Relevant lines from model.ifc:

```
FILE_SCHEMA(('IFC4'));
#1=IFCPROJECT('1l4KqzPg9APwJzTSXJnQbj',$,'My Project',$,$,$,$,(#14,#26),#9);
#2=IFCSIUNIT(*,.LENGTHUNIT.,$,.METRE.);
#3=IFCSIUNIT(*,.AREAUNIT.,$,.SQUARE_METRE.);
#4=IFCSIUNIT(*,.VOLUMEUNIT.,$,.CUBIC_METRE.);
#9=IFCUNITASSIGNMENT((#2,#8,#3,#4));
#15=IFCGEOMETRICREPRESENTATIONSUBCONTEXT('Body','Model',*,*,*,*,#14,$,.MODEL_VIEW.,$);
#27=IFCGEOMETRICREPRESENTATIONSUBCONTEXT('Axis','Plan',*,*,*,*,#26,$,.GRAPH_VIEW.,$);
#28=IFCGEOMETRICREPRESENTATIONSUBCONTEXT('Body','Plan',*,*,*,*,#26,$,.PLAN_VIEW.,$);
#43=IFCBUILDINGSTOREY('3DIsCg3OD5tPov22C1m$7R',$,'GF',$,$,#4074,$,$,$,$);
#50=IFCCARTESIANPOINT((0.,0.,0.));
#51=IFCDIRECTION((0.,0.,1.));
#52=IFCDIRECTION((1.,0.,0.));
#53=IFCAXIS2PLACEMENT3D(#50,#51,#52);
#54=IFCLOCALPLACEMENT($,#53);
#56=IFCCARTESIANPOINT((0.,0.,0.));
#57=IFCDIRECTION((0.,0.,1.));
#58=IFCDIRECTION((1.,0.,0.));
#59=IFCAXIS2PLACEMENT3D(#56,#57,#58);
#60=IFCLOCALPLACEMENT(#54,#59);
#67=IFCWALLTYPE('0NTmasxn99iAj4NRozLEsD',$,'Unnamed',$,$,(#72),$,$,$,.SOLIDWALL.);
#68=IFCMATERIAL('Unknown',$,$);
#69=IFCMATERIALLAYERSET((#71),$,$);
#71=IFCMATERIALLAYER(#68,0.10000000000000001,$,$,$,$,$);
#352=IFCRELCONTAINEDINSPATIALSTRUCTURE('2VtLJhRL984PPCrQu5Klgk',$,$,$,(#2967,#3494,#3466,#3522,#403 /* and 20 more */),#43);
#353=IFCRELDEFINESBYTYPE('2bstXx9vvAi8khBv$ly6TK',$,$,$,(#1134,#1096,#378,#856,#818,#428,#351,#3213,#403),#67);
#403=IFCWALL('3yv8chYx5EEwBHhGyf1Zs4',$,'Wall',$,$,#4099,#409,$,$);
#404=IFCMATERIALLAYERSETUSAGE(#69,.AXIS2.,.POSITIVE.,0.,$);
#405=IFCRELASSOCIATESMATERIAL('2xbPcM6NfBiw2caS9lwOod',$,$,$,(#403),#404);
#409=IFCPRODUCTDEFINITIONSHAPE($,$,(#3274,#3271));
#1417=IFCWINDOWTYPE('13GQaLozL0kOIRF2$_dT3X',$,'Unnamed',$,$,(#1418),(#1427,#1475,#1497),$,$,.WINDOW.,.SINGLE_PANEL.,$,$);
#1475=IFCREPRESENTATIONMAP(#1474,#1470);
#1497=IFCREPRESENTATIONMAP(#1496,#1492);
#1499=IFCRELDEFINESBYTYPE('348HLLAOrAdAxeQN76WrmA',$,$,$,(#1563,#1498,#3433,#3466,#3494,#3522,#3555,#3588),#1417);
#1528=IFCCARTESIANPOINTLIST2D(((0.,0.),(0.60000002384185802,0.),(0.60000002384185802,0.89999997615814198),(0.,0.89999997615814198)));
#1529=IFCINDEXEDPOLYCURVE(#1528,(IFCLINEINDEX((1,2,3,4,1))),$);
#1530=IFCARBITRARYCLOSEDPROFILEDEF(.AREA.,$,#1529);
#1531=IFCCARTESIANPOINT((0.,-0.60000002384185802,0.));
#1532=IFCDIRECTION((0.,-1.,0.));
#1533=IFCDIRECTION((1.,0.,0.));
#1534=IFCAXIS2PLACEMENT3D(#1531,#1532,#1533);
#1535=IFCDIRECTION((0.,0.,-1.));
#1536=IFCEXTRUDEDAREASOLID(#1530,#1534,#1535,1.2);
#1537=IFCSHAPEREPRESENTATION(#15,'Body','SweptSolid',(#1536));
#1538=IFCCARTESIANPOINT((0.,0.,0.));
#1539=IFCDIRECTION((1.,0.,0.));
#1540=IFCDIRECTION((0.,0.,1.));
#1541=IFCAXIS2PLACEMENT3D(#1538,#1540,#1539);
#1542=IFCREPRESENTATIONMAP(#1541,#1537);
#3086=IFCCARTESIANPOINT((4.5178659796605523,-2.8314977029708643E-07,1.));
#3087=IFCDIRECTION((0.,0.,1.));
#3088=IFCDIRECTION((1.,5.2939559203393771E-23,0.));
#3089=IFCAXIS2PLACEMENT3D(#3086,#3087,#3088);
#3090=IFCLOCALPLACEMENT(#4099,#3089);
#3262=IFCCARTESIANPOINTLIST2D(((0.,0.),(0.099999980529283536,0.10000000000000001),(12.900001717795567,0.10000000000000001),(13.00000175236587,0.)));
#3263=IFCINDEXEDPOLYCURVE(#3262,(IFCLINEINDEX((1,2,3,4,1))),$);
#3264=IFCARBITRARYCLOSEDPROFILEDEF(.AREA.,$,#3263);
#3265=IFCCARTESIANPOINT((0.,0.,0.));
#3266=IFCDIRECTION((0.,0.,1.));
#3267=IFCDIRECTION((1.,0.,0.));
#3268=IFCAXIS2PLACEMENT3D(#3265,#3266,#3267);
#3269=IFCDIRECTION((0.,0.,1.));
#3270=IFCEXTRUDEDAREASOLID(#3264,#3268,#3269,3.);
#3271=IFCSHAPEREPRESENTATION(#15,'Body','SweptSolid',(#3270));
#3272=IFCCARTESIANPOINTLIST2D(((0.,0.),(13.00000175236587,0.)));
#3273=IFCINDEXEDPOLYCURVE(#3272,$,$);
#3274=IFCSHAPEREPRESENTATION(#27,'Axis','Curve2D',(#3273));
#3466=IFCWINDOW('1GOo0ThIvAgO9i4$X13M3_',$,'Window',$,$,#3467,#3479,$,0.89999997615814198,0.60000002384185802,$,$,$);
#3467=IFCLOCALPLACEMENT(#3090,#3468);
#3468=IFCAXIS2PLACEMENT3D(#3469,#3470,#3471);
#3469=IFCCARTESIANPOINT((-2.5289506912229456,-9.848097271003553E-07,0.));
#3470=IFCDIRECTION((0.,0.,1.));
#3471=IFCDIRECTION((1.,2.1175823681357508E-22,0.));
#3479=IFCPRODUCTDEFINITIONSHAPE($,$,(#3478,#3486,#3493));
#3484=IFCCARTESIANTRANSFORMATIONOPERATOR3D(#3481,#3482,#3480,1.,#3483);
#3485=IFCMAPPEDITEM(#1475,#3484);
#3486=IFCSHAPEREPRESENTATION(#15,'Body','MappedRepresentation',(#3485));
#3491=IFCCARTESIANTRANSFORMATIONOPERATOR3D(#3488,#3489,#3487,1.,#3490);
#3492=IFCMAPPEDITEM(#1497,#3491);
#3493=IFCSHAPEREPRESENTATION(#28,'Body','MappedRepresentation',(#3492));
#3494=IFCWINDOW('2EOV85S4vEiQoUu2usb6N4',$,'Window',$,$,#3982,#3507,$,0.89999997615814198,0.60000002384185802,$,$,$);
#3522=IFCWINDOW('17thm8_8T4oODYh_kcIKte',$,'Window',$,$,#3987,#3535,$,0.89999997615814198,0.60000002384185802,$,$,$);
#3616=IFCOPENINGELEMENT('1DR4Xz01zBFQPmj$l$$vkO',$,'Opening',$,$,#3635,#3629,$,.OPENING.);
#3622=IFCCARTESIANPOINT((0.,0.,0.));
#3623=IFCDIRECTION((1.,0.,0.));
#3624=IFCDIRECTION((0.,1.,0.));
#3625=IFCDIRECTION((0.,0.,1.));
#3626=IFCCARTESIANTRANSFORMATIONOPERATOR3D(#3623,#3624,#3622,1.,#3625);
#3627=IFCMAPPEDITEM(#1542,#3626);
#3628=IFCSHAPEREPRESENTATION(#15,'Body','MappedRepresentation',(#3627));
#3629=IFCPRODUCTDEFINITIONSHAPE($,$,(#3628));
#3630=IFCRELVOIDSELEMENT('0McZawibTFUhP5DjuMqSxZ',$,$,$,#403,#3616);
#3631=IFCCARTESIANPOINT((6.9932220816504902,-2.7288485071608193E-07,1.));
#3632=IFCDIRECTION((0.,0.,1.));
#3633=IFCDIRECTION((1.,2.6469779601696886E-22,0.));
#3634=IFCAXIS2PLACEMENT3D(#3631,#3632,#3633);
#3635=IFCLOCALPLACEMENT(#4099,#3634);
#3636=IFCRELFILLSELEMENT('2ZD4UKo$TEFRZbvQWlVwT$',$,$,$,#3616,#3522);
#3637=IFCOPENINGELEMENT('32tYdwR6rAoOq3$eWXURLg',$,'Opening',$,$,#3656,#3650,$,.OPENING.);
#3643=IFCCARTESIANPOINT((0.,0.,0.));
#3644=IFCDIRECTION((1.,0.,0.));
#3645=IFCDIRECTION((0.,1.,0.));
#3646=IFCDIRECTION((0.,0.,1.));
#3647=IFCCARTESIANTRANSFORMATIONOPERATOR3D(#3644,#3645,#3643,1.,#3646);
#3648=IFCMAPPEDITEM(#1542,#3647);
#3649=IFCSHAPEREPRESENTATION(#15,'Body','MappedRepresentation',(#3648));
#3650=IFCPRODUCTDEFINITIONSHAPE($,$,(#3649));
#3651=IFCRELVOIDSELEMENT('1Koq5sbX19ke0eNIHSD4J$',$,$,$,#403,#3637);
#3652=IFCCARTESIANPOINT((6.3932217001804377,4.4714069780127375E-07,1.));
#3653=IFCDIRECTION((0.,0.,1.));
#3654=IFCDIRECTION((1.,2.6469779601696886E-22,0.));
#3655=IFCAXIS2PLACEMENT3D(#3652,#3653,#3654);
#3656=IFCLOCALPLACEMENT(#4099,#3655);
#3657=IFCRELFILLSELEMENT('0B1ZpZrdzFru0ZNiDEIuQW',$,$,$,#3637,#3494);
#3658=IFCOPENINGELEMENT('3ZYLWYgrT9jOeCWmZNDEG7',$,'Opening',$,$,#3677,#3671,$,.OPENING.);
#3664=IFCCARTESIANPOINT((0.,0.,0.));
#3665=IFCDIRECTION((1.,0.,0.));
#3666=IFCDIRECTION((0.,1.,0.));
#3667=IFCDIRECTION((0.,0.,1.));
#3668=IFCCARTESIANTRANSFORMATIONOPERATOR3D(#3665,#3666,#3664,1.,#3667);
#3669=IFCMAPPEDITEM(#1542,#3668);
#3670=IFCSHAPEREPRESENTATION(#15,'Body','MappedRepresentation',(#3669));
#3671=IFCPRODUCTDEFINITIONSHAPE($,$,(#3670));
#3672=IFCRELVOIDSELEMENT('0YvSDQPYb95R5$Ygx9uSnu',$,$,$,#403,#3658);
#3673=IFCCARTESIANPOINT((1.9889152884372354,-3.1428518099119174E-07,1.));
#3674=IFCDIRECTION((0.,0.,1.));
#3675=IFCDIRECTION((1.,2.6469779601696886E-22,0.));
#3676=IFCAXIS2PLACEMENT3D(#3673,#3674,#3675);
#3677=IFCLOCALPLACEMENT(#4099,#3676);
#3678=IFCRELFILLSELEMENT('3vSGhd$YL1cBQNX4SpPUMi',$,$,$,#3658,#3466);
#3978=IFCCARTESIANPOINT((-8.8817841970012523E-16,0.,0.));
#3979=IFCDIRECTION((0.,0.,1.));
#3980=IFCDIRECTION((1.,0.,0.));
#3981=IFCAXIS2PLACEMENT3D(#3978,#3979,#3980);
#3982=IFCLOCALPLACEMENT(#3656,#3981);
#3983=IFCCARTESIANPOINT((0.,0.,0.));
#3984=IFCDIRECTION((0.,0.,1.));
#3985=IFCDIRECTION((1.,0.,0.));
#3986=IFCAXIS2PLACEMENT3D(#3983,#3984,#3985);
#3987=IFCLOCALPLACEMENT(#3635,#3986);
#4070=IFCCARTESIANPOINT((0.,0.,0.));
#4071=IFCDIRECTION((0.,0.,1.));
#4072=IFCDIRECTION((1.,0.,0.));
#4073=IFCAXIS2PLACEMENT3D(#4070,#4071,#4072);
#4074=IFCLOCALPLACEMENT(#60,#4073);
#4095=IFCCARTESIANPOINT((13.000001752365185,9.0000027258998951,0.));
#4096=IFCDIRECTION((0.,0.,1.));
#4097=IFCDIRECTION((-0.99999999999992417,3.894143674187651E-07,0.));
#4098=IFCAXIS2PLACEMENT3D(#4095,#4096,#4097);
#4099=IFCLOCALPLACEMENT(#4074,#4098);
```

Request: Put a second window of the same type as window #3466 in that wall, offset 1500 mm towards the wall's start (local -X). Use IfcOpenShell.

```python
import ifcopenshell
import ifcopenshell.api.feature
import ifcopenshell.api.geometry
import ifcopenshell.api.root
import ifcopenshell.geom
import ifcopenshell.util.element
import ifcopenshell.util.placement
import ifcopenshell.util.shape
import ifcopenshell.util.unit

model = ifcopenshell.open("model.ifc")
unit_scale = ifcopenshell.util.unit.calculate_unit_scale(model)
settings = ifcopenshell.geom.settings()


def volume(element):
    """Net volume in cubic metres, openings subtracted."""
    shape = ifcopenshell.geom.create_shape(settings, element)
    return ifcopenshell.util.shape.get_volume(shape.geometry)


window = model.by_guid("1GOo0ThIvAgO9i4$X13M3_")
opening = window.FillsVoids[0].RelatingOpeningElement
wall = opening.VoidsElements[0].RelatingBuildingElement
before = volume(wall)
shift = ifcopenshell.util.placement.get_local_placement(wall.ObjectPlacement)[:3, 0] * -1.5 / unit_scale

# copy_class copies the void relationship, type, container and properties, but no geometry.
new_opening = ifcopenshell.api.root.copy_class(model, product=opening)
new_opening.Representation = ifcopenshell.util.element.copy_deep(
    model, opening.Representation, exclude=["IfcGeometricRepresentationContext", "IfcRepresentationMap"]
)
new_window = ifcopenshell.api.root.copy_class(model, product=window)
new_window.Representation = ifcopenshell.util.element.copy_deep(
    model, window.Representation, exclude=["IfcGeometricRepresentationContext", "IfcRepresentationMap"]
)
ifcopenshell.api.feature.add_filling(model, opening=new_opening, element=new_window)

for old, new in ((opening, new_opening), (window, new_window)):
    matrix = ifcopenshell.util.placement.get_local_placement(old.ObjectPlacement)
    matrix[:3, 3] += shift
    ifcopenshell.api.geometry.edit_object_placement(model, product=new, matrix=matrix, is_si=False)

after = volume(wall)

print(f"wall volume {before:.3f} -> {after:.3f} m3")

model.write("model_rev.ifc")
```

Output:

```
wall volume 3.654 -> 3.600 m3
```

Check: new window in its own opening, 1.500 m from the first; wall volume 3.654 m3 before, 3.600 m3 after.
